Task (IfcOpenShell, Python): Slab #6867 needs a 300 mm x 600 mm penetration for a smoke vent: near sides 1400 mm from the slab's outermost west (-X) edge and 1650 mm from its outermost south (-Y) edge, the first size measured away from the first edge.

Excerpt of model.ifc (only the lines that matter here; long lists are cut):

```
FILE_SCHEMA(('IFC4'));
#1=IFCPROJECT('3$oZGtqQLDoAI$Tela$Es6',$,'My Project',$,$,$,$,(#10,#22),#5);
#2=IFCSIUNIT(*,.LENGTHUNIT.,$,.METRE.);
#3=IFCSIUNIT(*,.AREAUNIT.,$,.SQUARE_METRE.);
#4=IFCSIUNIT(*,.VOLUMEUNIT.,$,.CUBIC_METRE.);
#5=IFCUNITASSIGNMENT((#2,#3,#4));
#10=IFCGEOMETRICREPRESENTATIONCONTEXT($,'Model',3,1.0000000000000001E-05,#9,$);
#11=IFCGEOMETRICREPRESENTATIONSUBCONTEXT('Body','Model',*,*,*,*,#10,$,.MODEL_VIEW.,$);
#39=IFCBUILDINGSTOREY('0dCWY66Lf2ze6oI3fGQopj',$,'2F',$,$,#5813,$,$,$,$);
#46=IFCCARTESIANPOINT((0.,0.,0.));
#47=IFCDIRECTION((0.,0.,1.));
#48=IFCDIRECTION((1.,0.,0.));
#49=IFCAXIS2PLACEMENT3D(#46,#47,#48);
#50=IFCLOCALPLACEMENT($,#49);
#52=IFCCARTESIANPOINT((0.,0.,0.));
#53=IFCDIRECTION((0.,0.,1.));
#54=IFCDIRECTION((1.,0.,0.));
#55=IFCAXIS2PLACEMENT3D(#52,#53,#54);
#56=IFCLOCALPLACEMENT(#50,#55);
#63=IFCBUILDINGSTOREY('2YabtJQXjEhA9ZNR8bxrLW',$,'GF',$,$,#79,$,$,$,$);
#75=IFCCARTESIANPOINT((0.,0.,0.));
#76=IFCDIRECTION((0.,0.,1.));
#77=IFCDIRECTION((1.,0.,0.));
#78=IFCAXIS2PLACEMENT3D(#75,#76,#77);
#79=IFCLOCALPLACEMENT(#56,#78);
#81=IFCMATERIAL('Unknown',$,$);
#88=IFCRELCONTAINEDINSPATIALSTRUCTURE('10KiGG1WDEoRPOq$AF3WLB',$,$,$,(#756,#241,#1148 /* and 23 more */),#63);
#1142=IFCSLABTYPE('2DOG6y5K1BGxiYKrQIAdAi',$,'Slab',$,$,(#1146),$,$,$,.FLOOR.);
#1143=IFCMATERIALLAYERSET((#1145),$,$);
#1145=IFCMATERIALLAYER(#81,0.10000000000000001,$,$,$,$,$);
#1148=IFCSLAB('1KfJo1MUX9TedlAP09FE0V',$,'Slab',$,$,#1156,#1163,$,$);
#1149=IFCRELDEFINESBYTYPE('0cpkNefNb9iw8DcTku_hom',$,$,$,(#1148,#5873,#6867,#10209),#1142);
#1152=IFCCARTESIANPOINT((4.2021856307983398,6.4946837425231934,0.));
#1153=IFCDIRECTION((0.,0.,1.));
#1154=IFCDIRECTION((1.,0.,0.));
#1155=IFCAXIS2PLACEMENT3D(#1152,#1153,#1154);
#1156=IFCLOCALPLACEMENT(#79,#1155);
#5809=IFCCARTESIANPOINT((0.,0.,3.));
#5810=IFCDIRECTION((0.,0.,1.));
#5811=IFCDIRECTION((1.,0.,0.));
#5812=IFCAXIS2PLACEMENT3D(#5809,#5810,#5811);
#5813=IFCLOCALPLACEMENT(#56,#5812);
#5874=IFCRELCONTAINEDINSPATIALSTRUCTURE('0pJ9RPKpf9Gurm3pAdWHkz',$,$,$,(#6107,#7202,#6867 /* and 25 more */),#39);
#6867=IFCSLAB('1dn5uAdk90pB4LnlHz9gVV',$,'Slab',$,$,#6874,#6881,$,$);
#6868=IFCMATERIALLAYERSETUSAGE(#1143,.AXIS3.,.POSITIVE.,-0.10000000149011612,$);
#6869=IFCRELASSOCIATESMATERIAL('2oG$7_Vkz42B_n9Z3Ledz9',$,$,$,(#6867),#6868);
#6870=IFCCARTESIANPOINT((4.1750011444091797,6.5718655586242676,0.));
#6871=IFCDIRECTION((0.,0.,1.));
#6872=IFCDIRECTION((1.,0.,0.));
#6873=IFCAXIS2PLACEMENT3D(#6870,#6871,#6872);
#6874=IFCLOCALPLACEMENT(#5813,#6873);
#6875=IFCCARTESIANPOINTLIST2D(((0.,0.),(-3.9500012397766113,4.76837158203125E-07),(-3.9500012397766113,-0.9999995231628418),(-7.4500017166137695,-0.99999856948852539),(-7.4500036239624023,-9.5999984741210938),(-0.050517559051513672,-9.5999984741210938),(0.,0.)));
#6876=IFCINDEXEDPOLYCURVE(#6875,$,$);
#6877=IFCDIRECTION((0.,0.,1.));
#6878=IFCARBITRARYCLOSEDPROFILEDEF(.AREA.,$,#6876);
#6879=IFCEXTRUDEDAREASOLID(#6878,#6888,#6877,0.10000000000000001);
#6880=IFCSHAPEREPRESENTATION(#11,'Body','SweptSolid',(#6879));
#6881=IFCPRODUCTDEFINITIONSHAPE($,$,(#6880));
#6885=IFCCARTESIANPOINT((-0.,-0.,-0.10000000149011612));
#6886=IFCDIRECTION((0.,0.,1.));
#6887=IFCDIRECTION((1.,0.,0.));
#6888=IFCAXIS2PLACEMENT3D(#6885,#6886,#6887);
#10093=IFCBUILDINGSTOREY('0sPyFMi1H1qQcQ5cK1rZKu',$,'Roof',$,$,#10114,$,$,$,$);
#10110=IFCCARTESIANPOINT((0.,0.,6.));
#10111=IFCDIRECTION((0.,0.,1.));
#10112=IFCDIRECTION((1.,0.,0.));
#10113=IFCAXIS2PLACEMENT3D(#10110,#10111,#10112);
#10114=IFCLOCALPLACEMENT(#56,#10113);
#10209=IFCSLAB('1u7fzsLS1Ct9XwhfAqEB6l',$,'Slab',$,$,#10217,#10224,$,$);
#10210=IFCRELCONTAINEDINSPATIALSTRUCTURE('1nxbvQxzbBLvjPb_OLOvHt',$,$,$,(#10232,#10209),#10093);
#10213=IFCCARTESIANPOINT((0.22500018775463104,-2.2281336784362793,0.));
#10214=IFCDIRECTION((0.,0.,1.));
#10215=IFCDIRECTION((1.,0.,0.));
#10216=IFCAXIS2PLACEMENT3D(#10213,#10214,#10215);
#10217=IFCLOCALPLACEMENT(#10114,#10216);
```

```python
import numpy as np
import ifcopenshell
import ifcopenshell.api.feature
import ifcopenshell.api.geometry
import ifcopenshell.api.root
import ifcopenshell.geom
import ifcopenshell.util.placement
import ifcopenshell.util.representation
import ifcopenshell.util.shape
import ifcopenshell.util.unit

model = ifcopenshell.open("model.ifc")
unit_scale = ifcopenshell.util.unit.calculate_unit_scale(model)
settings = ifcopenshell.geom.settings()


def volume(element):
    """Net volume in cubic metres, openings subtracted."""
    shape = ifcopenshell.geom.create_shape(settings, element)
    return ifcopenshell.util.shape.get_volume(shape.geometry)


slab = model.by_guid("1dn5uAdk90pB4LnlHz9gVV")
before = volume(slab)

# Extent in the slab's own axes, in metres. The edges named are its -X and -Y sides.
slab_shape = ifcopenshell.geom.create_shape(settings, slab)
vertices = ifcopenshell.util.shape.get_vertices(slab_shape.geometry)
x_min, y_min, bottom = vertices.min(axis=0)
top = vertices[:, 2].max()

opening = ifcopenshell.api.root.create_entity(model, ifc_class="IfcOpeningElement", name="Smoke vent opening", predefined_type="OPENING")
context = ifcopenshell.util.representation.get_context(model, "Model", "Body", "MODEL_VIEW")
width, depth = 0.3, 0.6
outline = [(0.0, 0.0), (width, 0.0), (width, depth), (0.0, depth), (0.0, 0.0)]
# Overshoot both faces by 50 mm so the cut is clean.
shape = ifcopenshell.api.geometry.add_slab_representation(
    model, context=context, depth=top - bottom + 0.1, polyline=outline
)
ifcopenshell.api.geometry.assign_representation(model, product=opening, representation=shape)

matrix = ifcopenshell.util.placement.get_local_placement(slab.ObjectPlacement)
matrix[:, 3] = matrix @ np.append(np.array([x_min + 1.4, y_min + 1.65, bottom - 0.05]) / unit_scale, 1.0)
ifcopenshell.api.geometry.edit_object_placement(model, product=opening, matrix=matrix, is_si=False)
ifcopenshell.api.feature.add_feature(model, feature=opening, element=slab)

after = volume(slab)

print(f"slab volume {before:.3f} -> {after:.3f} m3")

model.write("model_edited.ifc")
```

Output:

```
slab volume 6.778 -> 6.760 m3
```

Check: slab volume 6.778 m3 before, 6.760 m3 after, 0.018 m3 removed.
